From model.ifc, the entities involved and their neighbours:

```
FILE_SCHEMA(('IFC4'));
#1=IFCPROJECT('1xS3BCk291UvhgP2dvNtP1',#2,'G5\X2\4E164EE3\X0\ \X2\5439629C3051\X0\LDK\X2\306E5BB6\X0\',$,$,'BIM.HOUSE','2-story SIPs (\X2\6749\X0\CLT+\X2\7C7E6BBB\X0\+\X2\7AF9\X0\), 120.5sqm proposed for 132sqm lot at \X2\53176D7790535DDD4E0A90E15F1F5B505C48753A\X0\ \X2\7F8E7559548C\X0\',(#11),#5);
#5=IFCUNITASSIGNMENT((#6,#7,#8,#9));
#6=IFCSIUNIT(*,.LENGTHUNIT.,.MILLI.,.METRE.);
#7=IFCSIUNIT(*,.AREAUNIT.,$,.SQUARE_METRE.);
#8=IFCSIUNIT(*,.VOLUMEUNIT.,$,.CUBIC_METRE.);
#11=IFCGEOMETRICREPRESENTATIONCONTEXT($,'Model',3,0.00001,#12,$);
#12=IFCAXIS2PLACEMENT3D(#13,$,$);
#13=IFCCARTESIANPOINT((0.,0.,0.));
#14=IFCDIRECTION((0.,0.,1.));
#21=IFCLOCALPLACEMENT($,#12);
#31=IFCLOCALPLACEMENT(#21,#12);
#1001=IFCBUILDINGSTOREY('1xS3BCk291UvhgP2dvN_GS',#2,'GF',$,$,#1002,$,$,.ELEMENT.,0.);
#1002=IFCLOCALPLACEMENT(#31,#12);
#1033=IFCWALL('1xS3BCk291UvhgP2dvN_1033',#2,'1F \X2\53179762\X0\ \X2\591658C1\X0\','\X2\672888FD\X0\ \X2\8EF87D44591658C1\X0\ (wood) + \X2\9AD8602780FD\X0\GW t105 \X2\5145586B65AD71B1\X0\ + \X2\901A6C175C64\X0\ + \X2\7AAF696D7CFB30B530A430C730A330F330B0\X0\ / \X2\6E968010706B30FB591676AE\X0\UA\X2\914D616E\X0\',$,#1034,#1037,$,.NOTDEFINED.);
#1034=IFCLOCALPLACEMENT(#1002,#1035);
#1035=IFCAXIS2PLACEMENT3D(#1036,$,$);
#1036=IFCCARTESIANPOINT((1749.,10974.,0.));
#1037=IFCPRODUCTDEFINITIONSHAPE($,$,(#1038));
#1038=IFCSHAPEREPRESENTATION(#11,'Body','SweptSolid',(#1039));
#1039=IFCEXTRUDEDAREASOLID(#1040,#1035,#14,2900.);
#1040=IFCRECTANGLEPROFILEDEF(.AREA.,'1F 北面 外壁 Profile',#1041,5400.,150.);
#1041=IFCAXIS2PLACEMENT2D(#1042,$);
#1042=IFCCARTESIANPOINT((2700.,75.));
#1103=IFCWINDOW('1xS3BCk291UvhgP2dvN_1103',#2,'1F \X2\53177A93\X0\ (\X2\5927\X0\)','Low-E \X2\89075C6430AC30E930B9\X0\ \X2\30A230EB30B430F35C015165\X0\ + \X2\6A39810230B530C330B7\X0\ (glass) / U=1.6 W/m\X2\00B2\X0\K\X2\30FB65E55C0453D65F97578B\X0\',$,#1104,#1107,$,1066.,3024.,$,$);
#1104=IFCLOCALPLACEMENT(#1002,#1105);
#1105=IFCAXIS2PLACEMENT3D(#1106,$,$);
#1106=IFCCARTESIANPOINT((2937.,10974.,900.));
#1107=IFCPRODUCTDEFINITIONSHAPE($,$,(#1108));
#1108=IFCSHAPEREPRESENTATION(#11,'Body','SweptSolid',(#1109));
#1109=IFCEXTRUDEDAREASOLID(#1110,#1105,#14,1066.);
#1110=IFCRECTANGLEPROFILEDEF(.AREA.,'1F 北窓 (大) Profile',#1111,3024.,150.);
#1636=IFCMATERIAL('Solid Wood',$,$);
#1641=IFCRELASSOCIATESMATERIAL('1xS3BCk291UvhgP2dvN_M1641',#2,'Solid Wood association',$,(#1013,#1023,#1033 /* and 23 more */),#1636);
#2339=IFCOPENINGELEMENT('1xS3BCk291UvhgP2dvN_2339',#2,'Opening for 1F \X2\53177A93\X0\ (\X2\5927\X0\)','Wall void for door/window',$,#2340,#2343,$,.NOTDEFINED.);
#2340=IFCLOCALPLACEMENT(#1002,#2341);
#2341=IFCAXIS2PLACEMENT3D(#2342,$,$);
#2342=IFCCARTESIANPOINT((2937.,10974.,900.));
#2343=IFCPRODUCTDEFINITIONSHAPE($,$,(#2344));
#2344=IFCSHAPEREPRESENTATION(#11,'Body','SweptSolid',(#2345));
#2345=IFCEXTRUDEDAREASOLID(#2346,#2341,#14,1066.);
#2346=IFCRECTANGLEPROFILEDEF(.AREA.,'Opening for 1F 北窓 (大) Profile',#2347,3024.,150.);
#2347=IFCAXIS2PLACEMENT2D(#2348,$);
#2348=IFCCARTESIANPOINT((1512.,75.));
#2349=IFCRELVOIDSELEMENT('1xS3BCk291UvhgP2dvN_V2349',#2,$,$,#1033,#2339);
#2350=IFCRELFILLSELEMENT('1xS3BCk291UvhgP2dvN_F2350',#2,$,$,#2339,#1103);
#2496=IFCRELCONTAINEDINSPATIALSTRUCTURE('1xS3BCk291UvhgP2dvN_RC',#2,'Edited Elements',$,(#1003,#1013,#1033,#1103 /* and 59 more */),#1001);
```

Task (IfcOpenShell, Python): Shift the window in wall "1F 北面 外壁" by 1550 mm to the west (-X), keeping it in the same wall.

```python
import ifcopenshell
import ifcopenshell.api.geometry
import ifcopenshell.util.placement

model = ifcopenshell.open("model.ifc")

window = model.by_id(1103)
opening = window.FillsVoids[0].RelatingOpeningElement
wall = opening.VoidsElements[0].RelatingBuildingElement

wall_matrix = ifcopenshell.util.placement.get_local_placement(wall.ObjectPlacement)
shift = wall_matrix[:3, 0] * -1550.0
before = ifcopenshell.util.placement.get_local_placement(window.ObjectPlacement)[:3, 3].copy()

# The window is not placed relative to its opening, so move both.
for product in (opening, window):
    matrix = ifcopenshell.util.placement.get_local_placement(product.ObjectPlacement)
    matrix[:3, 3] += shift
    ifcopenshell.api.geometry.edit_object_placement(model, product=product, matrix=matrix, is_si=False)

after = ifcopenshell.util.placement.get_local_placement(window.ObjectPlacement)[:3, 3]
print("window moved by", (after - before).round(3) + 0.0)

model.write("model-out.ifc")
```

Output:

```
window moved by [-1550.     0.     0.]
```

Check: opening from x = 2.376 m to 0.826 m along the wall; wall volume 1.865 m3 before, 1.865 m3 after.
